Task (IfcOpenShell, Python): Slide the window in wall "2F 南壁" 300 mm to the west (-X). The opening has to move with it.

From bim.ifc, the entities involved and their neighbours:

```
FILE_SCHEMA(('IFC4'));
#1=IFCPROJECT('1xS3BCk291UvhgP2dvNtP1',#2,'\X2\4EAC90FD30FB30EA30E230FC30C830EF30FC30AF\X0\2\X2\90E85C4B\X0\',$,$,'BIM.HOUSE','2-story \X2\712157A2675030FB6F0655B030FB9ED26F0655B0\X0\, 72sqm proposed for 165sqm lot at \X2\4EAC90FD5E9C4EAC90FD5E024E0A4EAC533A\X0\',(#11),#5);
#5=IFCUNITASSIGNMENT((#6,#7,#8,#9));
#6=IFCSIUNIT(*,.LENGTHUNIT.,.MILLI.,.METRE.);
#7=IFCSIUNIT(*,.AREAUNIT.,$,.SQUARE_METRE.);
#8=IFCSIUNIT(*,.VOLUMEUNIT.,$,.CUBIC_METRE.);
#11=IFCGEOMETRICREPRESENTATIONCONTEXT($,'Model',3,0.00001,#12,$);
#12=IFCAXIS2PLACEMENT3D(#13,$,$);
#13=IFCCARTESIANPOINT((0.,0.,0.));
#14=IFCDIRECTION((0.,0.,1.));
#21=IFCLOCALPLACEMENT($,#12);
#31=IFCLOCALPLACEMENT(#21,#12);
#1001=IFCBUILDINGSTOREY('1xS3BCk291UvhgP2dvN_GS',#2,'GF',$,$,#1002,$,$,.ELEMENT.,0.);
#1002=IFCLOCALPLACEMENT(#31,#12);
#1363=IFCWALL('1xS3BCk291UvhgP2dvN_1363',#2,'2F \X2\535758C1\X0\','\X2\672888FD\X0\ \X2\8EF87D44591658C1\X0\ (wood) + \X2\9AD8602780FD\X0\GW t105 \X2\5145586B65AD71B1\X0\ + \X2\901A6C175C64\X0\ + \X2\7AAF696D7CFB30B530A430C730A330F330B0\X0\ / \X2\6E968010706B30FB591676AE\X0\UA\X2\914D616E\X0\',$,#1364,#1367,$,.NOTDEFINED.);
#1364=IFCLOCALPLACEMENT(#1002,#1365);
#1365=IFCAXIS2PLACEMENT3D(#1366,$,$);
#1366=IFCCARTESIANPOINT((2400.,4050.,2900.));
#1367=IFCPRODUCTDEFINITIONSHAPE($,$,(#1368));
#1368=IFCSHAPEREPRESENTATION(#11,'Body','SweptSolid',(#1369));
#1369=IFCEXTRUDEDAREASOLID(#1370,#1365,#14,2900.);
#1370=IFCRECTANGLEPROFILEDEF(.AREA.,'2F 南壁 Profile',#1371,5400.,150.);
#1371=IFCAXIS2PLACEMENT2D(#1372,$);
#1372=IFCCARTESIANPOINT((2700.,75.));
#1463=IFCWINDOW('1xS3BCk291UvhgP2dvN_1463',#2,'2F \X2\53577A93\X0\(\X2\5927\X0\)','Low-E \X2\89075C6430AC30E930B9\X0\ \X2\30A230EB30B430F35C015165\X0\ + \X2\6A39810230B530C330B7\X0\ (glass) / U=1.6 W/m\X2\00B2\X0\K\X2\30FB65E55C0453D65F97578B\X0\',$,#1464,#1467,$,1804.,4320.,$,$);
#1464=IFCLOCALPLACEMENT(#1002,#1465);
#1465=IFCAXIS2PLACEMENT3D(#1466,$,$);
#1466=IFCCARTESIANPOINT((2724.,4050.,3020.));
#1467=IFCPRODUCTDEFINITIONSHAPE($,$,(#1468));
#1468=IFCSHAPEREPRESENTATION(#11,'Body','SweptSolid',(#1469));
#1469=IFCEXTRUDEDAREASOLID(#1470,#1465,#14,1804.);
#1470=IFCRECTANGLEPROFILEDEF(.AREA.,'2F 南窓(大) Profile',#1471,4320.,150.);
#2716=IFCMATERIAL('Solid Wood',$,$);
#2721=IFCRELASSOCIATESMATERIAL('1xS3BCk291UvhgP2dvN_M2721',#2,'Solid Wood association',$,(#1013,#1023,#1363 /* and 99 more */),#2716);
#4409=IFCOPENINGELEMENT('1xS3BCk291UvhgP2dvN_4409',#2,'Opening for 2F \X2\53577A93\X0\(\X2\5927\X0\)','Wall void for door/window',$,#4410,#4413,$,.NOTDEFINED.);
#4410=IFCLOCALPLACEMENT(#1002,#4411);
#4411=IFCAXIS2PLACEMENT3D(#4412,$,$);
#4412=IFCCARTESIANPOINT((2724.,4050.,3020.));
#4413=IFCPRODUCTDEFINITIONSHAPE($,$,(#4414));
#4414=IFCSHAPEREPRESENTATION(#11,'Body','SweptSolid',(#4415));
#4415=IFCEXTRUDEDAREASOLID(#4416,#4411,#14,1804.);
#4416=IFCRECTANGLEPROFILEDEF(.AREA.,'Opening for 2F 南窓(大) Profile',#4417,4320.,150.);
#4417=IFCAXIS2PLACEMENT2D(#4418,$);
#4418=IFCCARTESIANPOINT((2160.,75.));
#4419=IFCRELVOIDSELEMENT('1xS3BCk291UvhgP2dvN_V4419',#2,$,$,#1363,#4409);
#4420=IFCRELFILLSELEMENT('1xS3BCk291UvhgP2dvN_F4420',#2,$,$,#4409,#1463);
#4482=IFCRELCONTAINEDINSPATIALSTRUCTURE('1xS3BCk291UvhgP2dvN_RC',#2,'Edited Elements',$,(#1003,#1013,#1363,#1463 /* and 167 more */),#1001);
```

```python
import ifcopenshell
import ifcopenshell.api.geometry
import ifcopenshell.util.placement
import ifcopenshell.util.unit

model = ifcopenshell.open("bim.ifc")
unit_scale = ifcopenshell.util.unit.calculate_unit_scale(model)

window = model.by_id(1463)
opening = window.FillsVoids[0].RelatingOpeningElement
wall = opening.VoidsElements[0].RelatingBuildingElement

wall_matrix = ifcopenshell.util.placement.get_local_placement(wall.ObjectPlacement)
shift = wall_matrix[:3, 0] * -0.3 / unit_scale
before = ifcopenshell.util.placement.get_local_placement(window.ObjectPlacement)[:3, 3].copy()

# The window is not placed relative to its opening, so move both.
for product in (opening, window):
    matrix = ifcopenshell.util.placement.get_local_placement(product.ObjectPlacement)
    matrix[:3, 3] += shift
    ifcopenshell.api.geometry.edit_object_placement(model, product=product, matrix=matrix, is_si=False)

after = ifcopenshell.util.placement.get_local_placement(window.ObjectPlacement)[:3, 3]
print("window moved by", (after - before).round(3) + 0.0)

model.write("bim_edited.ifc")
```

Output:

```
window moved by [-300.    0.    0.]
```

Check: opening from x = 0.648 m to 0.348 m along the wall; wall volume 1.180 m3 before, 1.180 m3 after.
